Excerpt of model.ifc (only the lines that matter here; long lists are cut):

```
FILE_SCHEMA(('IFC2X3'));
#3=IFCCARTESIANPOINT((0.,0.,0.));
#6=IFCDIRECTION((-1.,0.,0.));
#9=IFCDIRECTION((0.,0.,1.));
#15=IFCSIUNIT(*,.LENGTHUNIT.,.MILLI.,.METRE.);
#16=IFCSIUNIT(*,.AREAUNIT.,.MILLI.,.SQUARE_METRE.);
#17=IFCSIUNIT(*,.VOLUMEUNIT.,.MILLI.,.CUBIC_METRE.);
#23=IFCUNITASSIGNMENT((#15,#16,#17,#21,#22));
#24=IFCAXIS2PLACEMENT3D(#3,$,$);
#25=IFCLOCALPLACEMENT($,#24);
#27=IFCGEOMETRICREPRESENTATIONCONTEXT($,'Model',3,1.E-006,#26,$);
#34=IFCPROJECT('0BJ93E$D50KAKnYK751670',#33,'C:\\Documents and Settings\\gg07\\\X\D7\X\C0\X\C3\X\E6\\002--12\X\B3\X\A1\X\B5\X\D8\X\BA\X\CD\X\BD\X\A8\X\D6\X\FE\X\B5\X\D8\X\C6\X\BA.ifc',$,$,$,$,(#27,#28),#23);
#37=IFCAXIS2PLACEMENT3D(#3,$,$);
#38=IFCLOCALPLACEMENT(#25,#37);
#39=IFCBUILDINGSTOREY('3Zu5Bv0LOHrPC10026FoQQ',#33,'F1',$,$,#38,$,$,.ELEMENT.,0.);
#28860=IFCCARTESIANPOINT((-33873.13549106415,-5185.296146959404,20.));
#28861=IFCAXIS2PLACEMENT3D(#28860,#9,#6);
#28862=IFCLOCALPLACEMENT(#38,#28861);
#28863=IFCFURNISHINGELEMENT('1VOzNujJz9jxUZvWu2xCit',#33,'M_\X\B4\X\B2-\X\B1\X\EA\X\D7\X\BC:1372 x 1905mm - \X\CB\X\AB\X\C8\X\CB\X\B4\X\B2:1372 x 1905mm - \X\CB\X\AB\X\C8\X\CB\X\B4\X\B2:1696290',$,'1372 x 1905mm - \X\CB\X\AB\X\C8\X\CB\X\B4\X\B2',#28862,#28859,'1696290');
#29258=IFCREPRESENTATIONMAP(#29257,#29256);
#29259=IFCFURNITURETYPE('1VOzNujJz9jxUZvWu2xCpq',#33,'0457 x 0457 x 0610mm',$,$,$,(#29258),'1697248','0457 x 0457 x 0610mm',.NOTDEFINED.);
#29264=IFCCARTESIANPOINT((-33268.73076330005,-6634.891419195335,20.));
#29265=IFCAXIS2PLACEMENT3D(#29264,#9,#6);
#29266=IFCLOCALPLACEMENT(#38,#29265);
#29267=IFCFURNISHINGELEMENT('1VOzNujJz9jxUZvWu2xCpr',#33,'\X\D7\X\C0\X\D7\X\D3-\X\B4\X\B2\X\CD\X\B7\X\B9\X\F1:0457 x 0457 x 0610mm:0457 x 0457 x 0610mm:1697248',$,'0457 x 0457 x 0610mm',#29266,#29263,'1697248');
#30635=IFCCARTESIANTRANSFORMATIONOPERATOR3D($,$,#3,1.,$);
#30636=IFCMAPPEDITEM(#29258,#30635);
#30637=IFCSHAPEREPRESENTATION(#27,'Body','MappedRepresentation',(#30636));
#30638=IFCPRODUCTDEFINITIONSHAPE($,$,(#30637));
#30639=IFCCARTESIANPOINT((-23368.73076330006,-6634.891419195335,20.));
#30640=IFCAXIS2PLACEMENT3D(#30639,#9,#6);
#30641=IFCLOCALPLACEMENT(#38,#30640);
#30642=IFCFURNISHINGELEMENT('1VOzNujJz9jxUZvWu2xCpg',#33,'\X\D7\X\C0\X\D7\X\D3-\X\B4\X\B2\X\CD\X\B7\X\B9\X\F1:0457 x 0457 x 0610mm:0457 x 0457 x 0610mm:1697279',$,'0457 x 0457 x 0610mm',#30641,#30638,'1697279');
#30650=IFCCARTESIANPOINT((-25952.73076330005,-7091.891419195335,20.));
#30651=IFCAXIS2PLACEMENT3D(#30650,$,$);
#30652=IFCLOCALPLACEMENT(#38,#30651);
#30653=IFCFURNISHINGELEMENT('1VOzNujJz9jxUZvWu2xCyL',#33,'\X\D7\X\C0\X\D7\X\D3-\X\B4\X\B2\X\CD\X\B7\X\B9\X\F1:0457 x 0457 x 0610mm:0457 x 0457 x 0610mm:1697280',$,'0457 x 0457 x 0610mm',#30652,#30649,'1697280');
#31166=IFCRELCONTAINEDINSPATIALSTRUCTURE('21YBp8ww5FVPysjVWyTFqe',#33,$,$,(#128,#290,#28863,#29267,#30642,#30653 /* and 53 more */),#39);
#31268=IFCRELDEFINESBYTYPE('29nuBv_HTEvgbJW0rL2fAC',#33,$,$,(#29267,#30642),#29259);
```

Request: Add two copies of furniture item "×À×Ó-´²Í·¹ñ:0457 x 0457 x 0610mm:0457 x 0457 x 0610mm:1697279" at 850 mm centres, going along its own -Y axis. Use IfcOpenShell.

```python
import ifcopenshell
import ifcopenshell.api.geometry
import ifcopenshell.api.root
import ifcopenshell.util.element
import ifcopenshell.util.placement

model = ifcopenshell.open("model.ifc")


def reuse_history(source, copy):
    """copy_class also copies each property set's owner history, people and application; keep the originals."""
    for rel in copy.IsDefinedBy:
        if rel.is_a("IfcRelDefinesByProperties") and (history := rel.RelatingPropertyDefinition.OwnerHistory):
            rel.RelatingPropertyDefinition.OwnerHistory = source.OwnerHistory
            ifcopenshell.util.element.remove_deep2(model, history)


source = model.by_guid("1VOzNujJz9jxUZvWu2xCpg")
base = ifcopenshell.util.placement.get_local_placement(source.ObjectPlacement)
step = -base[:3, 1] * 850.0

for i in range(1, 3):
    copy = ifcopenshell.api.root.copy_class(model, product=source)
    copy.Representation = ifcopenshell.util.element.copy_deep(
        model, source.Representation, exclude=["IfcGeometricRepresentationContext", "IfcRepresentationMap"]
    )
    copy.Name = "×À×Ó-´²Í·¹ñ:0457 x 0457 x 0610mm:0457 x 0457 x 0610mm"
    copy.Tag = None
    reuse_history(source, copy)
    matrix = base.copy()
    matrix[:3, 3] += i * step
    print("added at", matrix[:3, 3].round(3) + 0.0)
    ifcopenshell.api.geometry.edit_object_placement(model, product=copy, matrix=matrix, is_si=False)

model.write("model_edited.ifc")
```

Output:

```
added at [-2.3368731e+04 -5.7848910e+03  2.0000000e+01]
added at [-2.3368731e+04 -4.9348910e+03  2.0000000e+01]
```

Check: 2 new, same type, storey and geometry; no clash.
